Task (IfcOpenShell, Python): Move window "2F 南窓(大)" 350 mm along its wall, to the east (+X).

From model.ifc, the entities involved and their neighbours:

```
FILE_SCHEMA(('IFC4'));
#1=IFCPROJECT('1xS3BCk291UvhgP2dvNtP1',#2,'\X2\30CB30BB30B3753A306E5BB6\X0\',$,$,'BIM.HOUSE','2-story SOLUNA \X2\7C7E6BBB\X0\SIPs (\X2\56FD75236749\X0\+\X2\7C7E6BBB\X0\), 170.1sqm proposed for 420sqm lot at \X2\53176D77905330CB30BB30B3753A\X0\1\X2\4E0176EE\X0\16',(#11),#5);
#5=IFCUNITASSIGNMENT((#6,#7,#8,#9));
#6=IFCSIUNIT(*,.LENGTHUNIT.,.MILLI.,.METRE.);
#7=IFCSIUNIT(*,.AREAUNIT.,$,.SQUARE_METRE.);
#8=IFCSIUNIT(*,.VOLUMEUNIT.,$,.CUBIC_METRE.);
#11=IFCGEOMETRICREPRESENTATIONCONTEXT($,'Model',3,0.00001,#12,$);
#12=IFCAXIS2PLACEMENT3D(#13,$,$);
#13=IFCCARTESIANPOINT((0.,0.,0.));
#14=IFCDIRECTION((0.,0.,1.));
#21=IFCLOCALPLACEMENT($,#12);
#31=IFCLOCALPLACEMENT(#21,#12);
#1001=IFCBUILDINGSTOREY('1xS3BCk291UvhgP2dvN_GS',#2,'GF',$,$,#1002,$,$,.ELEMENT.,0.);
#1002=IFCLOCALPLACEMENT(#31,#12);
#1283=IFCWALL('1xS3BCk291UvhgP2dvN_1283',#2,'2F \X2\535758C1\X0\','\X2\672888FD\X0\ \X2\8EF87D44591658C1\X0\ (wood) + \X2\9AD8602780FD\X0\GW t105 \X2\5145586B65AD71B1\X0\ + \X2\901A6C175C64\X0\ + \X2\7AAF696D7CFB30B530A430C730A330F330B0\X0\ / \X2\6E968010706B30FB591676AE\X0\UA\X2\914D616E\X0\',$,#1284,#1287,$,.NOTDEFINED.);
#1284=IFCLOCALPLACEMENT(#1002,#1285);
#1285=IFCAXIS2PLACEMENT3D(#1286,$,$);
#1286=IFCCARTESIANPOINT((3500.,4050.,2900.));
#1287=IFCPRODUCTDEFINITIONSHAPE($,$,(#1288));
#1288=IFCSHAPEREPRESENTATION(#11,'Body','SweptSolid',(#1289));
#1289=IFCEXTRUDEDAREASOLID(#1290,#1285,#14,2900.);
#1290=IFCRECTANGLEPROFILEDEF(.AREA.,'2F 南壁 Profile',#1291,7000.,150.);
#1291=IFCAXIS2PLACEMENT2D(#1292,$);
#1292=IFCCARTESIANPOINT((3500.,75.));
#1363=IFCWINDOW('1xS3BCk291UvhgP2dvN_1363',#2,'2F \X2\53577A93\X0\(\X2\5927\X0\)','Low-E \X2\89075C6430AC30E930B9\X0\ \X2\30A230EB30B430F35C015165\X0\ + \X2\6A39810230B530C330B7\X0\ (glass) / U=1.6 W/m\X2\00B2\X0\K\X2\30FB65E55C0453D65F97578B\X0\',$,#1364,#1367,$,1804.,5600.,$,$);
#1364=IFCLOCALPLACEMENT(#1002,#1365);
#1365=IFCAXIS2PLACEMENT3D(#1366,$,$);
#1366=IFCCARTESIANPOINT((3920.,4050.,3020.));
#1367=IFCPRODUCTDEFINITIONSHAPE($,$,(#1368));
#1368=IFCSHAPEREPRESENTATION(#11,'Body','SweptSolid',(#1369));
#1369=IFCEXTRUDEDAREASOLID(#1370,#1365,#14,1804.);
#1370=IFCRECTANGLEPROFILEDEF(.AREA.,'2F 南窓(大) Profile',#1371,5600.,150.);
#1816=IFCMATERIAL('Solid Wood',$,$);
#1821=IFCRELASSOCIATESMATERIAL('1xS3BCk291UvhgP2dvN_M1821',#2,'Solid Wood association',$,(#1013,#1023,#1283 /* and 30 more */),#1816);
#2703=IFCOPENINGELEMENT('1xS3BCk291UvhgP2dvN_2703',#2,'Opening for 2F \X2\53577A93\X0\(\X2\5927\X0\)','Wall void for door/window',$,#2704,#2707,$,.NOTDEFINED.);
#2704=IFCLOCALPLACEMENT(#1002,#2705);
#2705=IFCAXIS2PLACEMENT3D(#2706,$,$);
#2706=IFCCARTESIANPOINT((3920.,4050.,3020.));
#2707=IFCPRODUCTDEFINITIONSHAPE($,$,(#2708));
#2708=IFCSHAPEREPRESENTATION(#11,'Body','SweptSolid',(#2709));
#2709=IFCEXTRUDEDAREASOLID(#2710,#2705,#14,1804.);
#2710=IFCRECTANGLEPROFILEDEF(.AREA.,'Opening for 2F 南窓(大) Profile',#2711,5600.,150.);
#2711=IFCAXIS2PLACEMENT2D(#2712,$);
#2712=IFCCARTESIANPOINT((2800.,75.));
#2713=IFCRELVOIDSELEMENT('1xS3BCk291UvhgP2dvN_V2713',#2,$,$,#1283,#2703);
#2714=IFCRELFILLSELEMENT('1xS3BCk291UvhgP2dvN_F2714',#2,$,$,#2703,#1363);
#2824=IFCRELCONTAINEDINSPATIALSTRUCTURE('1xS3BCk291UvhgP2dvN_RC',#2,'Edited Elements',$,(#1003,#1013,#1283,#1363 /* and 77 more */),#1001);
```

```python
import ifcopenshell
import ifcopenshell.api.geometry
import ifcopenshell.util.placement
import ifcopenshell.util.unit

model = ifcopenshell.open("model.ifc")
unit_scale = ifcopenshell.util.unit.calculate_unit_scale(model)

window = model.by_id(1363)
opening = window.FillsVoids[0].RelatingOpeningElement
wall = opening.VoidsElements[0].RelatingBuildingElement

wall_matrix = ifcopenshell.util.placement.get_local_placement(wall.ObjectPlacement)
shift = wall_matrix[:3, 0] * 0.35 / unit_scale
before = ifcopenshell.util.placement.get_local_placement(window.ObjectPlacement)[:3, 3].copy()

# The window is not placed relative to its opening, so move both.
for product in (opening, window):
    matrix = ifcopenshell.util.placement.get_local_placement(product.ObjectPlacement)
    matrix[:3, 3] += shift
    ifcopenshell.api.geometry.edit_object_placement(model, product=product, matrix=matrix, is_si=False)

after = ifcopenshell.util.placement.get_local_placement(window.ObjectPlacement)[:3, 3]
print("window moved by", (after - before).round(3) + 0.0)

model.write("model-out.ifc")
```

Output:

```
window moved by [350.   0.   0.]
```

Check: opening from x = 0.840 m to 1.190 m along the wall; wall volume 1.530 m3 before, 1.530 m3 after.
